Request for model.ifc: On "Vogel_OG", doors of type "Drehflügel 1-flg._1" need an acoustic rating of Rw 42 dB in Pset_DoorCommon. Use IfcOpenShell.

First a look at what the model holds.

```python
import ifcopenshell
import ifcopenshell.util.element

model = ifcopenshell.open("model.ifc")
print(model.schema)
storey = next(s for s in model.by_type("IfcBuildingStorey") if s.Name == "Vogel_OG")
doors = [e for e in ifcopenshell.util.element.get_decomposition(storey) if e.is_a("IfcDoor")]
seen = {}
for e in doors:
    element_type = ifcopenshell.util.element.get_type(e)
    key = (element_type.Name if element_type != e and element_type else None, ifcopenshell.util.element.get_pset(e, "Pset_DoorCommon", "AcousticRating"))
    seen[key] = seen.get(key, 0) + 1
for (name, value), count in sorted(seen.items(), key=str):
    print(count, "x", name, "|", value)
```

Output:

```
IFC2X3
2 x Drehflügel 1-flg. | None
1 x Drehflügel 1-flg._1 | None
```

```python
import ifcopenshell
import ifcopenshell.api.pset
import ifcopenshell.util.element

model = ifcopenshell.open("model.ifc")

storey = next(s for s in model.by_type("IfcBuildingStorey") if s.Name == "Vogel_OG")
doors = [e for e in ifcopenshell.util.element.get_decomposition(storey) if e.is_a("IfcDoor")]

count = 0
for e in doors:
    element_type = ifcopenshell.util.element.get_type(e)
    if element_type in (None, e) or element_type.Name != "Drehflügel 1-flg._1":
        continue
    # add_pset returns the element's existing set when there is one.
    pset = ifcopenshell.api.pset.add_pset(model, product=e, name="Pset_DoorCommon")
    ifcopenshell.api.pset.edit_pset(model, pset=pset, properties={"AcousticRating": "Rw 42 dB"})
    count += 1

print(count, "doors updated")

model.write("model_v2.ifc")
```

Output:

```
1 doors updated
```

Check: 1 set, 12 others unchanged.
